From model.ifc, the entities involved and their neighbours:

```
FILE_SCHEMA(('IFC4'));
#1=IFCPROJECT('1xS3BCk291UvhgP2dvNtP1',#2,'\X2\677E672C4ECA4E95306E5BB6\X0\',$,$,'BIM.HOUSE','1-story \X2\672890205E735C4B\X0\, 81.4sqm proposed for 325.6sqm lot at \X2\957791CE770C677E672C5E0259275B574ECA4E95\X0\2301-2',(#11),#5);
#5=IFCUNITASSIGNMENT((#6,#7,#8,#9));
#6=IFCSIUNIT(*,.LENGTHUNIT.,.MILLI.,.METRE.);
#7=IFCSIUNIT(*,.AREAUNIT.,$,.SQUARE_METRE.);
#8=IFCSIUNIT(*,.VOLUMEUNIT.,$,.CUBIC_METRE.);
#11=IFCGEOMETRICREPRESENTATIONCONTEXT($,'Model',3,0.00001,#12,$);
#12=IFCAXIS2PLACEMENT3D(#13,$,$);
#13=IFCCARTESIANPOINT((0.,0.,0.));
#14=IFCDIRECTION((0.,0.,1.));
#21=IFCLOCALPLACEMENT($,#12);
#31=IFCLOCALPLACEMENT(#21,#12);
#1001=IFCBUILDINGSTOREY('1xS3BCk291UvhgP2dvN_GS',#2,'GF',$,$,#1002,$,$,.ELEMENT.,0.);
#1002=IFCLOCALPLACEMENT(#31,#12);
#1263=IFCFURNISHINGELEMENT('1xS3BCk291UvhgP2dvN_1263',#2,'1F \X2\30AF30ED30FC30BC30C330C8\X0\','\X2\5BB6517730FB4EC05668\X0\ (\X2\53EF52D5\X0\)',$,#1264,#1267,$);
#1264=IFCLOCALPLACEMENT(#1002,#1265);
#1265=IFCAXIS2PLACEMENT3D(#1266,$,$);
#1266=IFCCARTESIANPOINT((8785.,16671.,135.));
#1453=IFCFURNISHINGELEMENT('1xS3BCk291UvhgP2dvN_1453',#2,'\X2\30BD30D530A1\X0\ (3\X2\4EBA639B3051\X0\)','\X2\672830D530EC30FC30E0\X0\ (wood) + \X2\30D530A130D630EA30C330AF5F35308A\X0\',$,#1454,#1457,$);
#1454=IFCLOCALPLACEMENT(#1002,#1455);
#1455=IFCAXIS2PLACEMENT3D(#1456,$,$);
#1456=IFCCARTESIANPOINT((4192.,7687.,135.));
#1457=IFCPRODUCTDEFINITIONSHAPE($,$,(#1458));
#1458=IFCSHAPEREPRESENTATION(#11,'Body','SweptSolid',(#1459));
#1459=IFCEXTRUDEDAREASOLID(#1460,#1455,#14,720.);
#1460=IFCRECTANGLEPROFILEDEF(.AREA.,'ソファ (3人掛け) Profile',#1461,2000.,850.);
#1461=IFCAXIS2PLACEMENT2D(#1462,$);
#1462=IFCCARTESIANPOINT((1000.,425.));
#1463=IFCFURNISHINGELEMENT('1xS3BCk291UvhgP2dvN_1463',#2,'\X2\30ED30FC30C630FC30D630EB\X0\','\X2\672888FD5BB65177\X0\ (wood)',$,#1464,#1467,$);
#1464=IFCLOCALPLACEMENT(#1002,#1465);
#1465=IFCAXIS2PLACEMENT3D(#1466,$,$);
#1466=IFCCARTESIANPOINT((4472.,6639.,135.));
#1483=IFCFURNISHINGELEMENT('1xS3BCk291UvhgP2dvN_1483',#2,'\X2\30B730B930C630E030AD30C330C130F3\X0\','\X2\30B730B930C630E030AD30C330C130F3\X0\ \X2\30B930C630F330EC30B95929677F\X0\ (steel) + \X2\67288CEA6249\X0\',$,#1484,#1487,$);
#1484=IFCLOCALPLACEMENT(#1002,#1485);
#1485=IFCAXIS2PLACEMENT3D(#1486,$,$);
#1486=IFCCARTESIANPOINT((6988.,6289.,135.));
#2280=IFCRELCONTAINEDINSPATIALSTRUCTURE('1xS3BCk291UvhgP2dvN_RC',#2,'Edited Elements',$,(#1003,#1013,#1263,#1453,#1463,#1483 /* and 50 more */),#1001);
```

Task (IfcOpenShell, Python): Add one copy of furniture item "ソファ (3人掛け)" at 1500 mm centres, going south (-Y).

```python
import numpy as np
import ifcopenshell
import ifcopenshell.api.geometry
import ifcopenshell.api.root
import ifcopenshell.util.element
import ifcopenshell.util.placement

model = ifcopenshell.open("model.ifc")


def reuse_history(source, copy):
    """copy_class also copies each property set's owner history, people and application; keep the originals."""
    for rel in copy.IsDefinedBy:
        if rel.is_a("IfcRelDefinesByProperties") and (history := rel.RelatingPropertyDefinition.OwnerHistory):
            rel.RelatingPropertyDefinition.OwnerHistory = source.OwnerHistory
            ifcopenshell.util.element.remove_deep2(model, history)


source = model.by_guid("1xS3BCk291UvhgP2dvN_1453")
base = ifcopenshell.util.placement.get_local_placement(source.ObjectPlacement)
step = np.array([0.0, -1.0, 0.0]) * 1500.0

for i in range(1, 2):
    copy = ifcopenshell.api.root.copy_class(model, product=source)
    copy.Representation = ifcopenshell.util.element.copy_deep(
        model, source.Representation, exclude=["IfcGeometricRepresentationContext", "IfcRepresentationMap"]
    )
    reuse_history(source, copy)
    matrix = base.copy()
    matrix[:3, 3] += i * step
    print("added at", matrix[:3, 3].round(3) + 0.0)
    ifcopenshell.api.geometry.edit_object_placement(model, product=copy, matrix=matrix, is_si=False)

model.write("model_rev.ifc")
```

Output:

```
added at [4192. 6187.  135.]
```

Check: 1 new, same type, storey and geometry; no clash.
